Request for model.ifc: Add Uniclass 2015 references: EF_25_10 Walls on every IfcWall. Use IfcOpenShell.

First a look at what the model holds.

```python
import ifcopenshell

model = ifcopenshell.open("model.ifc")
print(model.schema)
print("classifications:", [c.Name for c in model.by_type("IfcClassification")])
for ifc_class in ("IfcDoor", "IfcRoof", "IfcStair", "IfcWall", "IfcWindow"):
    print(ifc_class, len(model.by_type(ifc_class)))
```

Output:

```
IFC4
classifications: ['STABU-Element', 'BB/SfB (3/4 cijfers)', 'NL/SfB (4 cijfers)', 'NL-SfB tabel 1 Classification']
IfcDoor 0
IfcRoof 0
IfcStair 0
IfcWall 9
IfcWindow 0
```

```python
import ifcopenshell
import ifcopenshell.api.classification

model = ifcopenshell.open("model.ifc")

system = ifcopenshell.api.classification.add_classification(model, classification="Uniclass 2015")

codes = {
    "IfcWall": ("EF_25_10", "Walls"),
}
for ifc_class, (code, name) in codes.items():
    products = model.by_type(ifc_class)
    ifcopenshell.api.classification.add_reference(
        model, products=products, classification=system, identification=code, name=name
    )
    print(code, len(products))

model.write("model-out.ifc")
```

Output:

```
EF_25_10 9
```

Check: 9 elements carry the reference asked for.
